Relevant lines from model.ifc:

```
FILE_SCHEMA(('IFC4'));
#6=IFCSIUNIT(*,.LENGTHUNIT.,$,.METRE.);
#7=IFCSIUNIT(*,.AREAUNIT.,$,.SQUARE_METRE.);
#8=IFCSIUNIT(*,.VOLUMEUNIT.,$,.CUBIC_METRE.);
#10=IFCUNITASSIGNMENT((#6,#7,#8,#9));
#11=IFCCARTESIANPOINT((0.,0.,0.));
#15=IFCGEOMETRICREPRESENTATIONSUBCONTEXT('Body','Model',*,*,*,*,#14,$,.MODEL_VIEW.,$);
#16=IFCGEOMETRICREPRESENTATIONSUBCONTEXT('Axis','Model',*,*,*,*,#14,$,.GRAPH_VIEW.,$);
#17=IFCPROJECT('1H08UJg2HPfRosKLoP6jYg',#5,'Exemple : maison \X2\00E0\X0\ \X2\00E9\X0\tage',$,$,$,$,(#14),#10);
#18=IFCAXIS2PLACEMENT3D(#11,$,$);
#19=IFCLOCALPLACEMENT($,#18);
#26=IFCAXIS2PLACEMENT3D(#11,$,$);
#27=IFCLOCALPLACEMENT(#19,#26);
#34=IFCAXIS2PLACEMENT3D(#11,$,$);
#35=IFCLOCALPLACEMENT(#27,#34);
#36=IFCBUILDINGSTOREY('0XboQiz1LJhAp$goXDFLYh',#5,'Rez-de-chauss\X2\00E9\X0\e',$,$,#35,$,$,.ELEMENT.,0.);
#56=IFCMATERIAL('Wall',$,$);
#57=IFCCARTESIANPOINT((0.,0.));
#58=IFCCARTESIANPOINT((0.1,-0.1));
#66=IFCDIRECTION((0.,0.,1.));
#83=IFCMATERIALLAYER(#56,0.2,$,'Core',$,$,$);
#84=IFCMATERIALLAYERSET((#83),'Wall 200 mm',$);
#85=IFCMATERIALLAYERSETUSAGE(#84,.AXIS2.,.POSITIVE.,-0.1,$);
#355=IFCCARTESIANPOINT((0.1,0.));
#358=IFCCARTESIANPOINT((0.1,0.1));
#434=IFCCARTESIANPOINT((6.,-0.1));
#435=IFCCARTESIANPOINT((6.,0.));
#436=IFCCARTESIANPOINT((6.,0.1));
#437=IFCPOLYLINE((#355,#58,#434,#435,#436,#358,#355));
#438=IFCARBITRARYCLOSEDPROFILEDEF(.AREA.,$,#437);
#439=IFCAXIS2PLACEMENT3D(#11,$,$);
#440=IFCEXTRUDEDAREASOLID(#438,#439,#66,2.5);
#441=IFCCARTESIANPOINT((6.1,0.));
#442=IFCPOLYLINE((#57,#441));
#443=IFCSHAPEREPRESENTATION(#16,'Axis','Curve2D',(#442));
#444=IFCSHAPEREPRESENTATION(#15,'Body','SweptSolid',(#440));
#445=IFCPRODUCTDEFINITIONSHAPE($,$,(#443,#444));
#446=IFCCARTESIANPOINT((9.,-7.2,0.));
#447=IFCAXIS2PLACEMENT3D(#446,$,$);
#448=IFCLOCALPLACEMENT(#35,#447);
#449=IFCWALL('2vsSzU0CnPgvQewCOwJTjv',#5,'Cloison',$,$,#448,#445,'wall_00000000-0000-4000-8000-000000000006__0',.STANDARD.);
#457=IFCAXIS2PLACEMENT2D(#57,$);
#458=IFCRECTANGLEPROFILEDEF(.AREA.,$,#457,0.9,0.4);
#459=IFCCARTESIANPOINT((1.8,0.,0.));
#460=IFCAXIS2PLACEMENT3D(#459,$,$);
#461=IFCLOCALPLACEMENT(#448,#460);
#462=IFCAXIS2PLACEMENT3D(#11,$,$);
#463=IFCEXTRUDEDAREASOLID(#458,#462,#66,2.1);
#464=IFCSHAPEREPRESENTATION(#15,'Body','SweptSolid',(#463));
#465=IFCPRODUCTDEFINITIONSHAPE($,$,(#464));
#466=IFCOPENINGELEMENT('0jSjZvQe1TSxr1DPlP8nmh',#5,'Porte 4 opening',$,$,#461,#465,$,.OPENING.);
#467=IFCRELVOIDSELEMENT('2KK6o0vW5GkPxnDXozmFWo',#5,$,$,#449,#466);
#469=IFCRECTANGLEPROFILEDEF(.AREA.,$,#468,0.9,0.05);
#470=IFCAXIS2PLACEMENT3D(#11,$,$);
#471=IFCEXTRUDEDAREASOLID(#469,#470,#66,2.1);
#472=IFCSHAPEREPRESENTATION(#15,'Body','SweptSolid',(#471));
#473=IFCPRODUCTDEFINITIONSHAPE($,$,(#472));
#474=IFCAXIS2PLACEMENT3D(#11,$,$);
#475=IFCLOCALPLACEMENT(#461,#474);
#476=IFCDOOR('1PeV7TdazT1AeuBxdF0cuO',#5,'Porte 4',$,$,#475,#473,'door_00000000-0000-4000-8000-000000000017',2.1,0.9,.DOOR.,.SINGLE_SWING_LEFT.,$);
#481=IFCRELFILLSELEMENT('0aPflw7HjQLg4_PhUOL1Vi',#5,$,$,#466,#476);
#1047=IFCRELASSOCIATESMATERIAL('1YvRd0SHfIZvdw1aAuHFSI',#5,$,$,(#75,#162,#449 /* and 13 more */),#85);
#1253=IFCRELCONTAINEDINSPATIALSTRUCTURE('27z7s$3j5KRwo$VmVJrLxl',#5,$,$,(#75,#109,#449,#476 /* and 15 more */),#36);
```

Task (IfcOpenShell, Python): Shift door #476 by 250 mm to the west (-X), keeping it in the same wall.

```python
import ifcopenshell
import ifcopenshell.api.geometry
import ifcopenshell.util.placement

model = ifcopenshell.open("model.ifc")

door = model.by_id(476)
opening = door.FillsVoids[0].RelatingOpeningElement
wall = opening.VoidsElements[0].RelatingBuildingElement

wall_matrix = ifcopenshell.util.placement.get_local_placement(wall.ObjectPlacement)
shift = wall_matrix[:3, 0] * -0.25
before = ifcopenshell.util.placement.get_local_placement(door.ObjectPlacement)[:3, 3].copy()

# The door is placed relative to its opening, so it follows when the opening moves.
matrix = ifcopenshell.util.placement.get_local_placement(opening.ObjectPlacement)
matrix[:3, 3] += shift
ifcopenshell.api.geometry.edit_object_placement(
    model, product=opening, matrix=matrix, is_si=False, should_transform_children=True
)

after = ifcopenshell.util.placement.get_local_placement(door.ObjectPlacement)[:3, 3]
print("door moved by", (after - before).round(3) + 0.0)

model.write("model_rev.ifc")
```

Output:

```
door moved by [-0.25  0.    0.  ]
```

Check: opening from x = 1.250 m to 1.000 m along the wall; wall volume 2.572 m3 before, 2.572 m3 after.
